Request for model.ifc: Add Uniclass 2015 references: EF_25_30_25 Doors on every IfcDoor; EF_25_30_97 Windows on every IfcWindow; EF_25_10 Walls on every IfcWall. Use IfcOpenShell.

First a look at what the model holds.

```python
import ifcopenshell

model = ifcopenshell.open("model.ifc")
print(model.schema)
print("classifications:", [c.Name for c in model.by_type("IfcClassification")])
for ifc_class in ("IfcDoor", "IfcRoof", "IfcStair", "IfcWall", "IfcWindow"):
    print(ifc_class, len(model.by_type(ifc_class)))
```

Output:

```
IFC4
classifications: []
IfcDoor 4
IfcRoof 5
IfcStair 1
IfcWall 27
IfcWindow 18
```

```python
import ifcopenshell
import ifcopenshell.api.classification

model = ifcopenshell.open("model.ifc")

system = ifcopenshell.api.classification.add_classification(model, classification="Uniclass 2015")

codes = {
    "IfcDoor": ("EF_25_30_25", "Doors"),
    "IfcWindow": ("EF_25_30_97", "Windows"),
    "IfcWall": ("EF_25_10", "Walls"),
}
for ifc_class, (code, name) in codes.items():
    products = model.by_type(ifc_class)
    ifcopenshell.api.classification.add_reference(
        model, products=products, classification=system, identification=code, name=name
    )
    print(code, len(products))

model.write("model_v2.ifc")
```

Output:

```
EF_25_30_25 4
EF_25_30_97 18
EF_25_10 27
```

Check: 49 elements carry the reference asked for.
